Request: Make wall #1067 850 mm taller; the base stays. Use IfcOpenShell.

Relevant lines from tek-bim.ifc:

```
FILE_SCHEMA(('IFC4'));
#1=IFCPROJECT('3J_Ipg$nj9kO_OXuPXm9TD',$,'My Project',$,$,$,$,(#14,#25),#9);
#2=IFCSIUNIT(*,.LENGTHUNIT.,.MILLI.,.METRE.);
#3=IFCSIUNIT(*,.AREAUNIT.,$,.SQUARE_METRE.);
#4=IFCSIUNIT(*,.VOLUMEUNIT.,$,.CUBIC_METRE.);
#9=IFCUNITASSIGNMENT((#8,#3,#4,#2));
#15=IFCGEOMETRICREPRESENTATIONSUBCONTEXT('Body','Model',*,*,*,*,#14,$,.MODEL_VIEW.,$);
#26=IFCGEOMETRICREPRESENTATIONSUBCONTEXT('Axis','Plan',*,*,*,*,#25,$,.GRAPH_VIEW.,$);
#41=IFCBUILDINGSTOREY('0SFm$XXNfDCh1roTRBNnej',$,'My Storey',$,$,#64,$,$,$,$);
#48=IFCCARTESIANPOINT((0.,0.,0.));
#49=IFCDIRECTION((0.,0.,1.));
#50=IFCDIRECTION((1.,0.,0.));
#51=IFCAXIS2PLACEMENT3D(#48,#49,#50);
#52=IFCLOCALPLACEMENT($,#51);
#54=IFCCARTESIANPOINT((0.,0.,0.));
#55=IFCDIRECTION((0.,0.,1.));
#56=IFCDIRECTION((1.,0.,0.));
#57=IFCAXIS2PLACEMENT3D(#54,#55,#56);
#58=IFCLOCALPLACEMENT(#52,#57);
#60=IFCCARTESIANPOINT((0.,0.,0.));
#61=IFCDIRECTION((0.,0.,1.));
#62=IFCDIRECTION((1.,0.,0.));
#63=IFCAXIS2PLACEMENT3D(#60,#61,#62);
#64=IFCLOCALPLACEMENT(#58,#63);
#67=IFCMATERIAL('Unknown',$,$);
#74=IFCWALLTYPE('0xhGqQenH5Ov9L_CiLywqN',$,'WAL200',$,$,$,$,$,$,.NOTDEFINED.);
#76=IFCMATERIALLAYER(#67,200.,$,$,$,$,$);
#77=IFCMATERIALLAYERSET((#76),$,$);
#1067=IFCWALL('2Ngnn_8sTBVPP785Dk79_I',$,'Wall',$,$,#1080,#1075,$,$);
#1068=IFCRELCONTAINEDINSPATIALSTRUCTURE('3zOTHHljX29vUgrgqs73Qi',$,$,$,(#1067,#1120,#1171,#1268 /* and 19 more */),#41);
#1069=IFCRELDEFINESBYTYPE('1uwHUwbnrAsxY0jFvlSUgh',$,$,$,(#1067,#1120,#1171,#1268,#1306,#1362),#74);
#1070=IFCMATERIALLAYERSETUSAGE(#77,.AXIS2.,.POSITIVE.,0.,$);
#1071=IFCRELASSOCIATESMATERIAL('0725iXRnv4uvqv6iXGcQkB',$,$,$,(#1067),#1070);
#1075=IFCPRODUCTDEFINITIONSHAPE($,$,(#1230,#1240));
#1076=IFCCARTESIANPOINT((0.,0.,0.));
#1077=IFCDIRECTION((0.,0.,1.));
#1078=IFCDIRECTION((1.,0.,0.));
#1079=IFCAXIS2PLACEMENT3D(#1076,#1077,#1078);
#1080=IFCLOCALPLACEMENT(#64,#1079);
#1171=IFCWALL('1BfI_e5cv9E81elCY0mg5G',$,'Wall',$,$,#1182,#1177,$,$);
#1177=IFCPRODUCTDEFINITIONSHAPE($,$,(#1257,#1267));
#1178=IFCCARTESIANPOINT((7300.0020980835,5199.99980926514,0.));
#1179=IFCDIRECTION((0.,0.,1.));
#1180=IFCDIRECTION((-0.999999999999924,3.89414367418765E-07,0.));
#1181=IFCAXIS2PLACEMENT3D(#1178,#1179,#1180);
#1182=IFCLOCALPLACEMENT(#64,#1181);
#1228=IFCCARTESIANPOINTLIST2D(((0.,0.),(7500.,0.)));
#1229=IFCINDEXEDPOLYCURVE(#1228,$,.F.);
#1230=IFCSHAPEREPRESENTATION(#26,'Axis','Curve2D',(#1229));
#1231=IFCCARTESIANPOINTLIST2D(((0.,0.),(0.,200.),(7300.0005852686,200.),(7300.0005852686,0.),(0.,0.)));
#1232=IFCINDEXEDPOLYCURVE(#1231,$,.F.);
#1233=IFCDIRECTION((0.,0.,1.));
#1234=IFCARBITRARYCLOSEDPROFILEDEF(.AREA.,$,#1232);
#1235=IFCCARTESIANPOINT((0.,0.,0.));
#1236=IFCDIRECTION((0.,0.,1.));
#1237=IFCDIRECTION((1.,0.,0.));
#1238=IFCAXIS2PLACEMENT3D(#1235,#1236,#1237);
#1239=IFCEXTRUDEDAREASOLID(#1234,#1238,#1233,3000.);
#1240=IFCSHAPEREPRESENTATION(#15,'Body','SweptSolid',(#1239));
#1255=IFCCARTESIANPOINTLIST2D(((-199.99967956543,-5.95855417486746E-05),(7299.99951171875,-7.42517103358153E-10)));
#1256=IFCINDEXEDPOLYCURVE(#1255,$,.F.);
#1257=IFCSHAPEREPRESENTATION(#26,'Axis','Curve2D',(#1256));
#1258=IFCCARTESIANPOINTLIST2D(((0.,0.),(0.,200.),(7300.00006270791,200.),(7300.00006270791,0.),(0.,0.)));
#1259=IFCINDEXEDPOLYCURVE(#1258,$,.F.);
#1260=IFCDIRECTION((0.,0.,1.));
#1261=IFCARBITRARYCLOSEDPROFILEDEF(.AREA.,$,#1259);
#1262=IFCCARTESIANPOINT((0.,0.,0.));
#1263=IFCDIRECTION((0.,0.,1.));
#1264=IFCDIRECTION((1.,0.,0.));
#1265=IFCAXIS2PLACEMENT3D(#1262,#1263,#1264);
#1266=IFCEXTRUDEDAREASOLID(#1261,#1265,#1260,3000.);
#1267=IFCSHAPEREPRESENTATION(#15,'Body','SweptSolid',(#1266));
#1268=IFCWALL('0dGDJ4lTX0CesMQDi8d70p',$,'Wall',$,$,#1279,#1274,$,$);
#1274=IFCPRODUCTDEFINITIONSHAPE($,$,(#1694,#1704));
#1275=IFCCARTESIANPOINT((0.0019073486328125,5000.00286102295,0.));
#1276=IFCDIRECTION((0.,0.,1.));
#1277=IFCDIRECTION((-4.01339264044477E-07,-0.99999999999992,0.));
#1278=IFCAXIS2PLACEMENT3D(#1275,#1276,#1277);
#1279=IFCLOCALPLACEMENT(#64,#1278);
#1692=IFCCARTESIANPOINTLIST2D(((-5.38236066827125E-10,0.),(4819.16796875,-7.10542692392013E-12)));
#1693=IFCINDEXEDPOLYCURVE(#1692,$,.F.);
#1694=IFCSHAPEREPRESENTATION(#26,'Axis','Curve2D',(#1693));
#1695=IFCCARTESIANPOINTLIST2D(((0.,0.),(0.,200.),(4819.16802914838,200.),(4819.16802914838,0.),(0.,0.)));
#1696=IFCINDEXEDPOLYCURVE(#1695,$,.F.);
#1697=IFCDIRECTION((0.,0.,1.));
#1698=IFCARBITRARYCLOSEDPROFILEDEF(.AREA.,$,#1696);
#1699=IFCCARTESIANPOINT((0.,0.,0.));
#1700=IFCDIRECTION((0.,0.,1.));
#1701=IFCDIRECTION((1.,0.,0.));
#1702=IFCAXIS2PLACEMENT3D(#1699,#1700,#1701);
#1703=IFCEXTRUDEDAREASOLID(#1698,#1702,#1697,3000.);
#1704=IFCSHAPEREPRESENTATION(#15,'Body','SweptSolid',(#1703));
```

```python
import ifcopenshell
import ifcopenshell.geom
import ifcopenshell.util.representation
import ifcopenshell.util.shape

model = ifcopenshell.open("tek-bim.ifc")
settings = ifcopenshell.geom.settings()


def volume(element):
    """Net volume in cubic metres, openings subtracted."""
    shape = ifcopenshell.geom.create_shape(settings, element)
    return ifcopenshell.util.shape.get_volume(shape.geometry)


wall = model.by_guid("2Ngnn_8sTBVPP785Dk79_I")
before = volume(wall)

body = ifcopenshell.util.representation.get_representation(wall, "Model", "Body")
solid = body.Items[0]
old_height = solid.Depth
solid.Depth += 850.0
after = volume(wall)

print(f"height {old_height:g} -> {solid.Depth:g}, volume {before:.3f} -> {after:.3f} m3")

model.write("tek-bim-out.ifc")
```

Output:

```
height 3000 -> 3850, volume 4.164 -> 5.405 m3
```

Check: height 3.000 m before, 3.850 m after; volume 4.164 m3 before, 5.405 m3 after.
